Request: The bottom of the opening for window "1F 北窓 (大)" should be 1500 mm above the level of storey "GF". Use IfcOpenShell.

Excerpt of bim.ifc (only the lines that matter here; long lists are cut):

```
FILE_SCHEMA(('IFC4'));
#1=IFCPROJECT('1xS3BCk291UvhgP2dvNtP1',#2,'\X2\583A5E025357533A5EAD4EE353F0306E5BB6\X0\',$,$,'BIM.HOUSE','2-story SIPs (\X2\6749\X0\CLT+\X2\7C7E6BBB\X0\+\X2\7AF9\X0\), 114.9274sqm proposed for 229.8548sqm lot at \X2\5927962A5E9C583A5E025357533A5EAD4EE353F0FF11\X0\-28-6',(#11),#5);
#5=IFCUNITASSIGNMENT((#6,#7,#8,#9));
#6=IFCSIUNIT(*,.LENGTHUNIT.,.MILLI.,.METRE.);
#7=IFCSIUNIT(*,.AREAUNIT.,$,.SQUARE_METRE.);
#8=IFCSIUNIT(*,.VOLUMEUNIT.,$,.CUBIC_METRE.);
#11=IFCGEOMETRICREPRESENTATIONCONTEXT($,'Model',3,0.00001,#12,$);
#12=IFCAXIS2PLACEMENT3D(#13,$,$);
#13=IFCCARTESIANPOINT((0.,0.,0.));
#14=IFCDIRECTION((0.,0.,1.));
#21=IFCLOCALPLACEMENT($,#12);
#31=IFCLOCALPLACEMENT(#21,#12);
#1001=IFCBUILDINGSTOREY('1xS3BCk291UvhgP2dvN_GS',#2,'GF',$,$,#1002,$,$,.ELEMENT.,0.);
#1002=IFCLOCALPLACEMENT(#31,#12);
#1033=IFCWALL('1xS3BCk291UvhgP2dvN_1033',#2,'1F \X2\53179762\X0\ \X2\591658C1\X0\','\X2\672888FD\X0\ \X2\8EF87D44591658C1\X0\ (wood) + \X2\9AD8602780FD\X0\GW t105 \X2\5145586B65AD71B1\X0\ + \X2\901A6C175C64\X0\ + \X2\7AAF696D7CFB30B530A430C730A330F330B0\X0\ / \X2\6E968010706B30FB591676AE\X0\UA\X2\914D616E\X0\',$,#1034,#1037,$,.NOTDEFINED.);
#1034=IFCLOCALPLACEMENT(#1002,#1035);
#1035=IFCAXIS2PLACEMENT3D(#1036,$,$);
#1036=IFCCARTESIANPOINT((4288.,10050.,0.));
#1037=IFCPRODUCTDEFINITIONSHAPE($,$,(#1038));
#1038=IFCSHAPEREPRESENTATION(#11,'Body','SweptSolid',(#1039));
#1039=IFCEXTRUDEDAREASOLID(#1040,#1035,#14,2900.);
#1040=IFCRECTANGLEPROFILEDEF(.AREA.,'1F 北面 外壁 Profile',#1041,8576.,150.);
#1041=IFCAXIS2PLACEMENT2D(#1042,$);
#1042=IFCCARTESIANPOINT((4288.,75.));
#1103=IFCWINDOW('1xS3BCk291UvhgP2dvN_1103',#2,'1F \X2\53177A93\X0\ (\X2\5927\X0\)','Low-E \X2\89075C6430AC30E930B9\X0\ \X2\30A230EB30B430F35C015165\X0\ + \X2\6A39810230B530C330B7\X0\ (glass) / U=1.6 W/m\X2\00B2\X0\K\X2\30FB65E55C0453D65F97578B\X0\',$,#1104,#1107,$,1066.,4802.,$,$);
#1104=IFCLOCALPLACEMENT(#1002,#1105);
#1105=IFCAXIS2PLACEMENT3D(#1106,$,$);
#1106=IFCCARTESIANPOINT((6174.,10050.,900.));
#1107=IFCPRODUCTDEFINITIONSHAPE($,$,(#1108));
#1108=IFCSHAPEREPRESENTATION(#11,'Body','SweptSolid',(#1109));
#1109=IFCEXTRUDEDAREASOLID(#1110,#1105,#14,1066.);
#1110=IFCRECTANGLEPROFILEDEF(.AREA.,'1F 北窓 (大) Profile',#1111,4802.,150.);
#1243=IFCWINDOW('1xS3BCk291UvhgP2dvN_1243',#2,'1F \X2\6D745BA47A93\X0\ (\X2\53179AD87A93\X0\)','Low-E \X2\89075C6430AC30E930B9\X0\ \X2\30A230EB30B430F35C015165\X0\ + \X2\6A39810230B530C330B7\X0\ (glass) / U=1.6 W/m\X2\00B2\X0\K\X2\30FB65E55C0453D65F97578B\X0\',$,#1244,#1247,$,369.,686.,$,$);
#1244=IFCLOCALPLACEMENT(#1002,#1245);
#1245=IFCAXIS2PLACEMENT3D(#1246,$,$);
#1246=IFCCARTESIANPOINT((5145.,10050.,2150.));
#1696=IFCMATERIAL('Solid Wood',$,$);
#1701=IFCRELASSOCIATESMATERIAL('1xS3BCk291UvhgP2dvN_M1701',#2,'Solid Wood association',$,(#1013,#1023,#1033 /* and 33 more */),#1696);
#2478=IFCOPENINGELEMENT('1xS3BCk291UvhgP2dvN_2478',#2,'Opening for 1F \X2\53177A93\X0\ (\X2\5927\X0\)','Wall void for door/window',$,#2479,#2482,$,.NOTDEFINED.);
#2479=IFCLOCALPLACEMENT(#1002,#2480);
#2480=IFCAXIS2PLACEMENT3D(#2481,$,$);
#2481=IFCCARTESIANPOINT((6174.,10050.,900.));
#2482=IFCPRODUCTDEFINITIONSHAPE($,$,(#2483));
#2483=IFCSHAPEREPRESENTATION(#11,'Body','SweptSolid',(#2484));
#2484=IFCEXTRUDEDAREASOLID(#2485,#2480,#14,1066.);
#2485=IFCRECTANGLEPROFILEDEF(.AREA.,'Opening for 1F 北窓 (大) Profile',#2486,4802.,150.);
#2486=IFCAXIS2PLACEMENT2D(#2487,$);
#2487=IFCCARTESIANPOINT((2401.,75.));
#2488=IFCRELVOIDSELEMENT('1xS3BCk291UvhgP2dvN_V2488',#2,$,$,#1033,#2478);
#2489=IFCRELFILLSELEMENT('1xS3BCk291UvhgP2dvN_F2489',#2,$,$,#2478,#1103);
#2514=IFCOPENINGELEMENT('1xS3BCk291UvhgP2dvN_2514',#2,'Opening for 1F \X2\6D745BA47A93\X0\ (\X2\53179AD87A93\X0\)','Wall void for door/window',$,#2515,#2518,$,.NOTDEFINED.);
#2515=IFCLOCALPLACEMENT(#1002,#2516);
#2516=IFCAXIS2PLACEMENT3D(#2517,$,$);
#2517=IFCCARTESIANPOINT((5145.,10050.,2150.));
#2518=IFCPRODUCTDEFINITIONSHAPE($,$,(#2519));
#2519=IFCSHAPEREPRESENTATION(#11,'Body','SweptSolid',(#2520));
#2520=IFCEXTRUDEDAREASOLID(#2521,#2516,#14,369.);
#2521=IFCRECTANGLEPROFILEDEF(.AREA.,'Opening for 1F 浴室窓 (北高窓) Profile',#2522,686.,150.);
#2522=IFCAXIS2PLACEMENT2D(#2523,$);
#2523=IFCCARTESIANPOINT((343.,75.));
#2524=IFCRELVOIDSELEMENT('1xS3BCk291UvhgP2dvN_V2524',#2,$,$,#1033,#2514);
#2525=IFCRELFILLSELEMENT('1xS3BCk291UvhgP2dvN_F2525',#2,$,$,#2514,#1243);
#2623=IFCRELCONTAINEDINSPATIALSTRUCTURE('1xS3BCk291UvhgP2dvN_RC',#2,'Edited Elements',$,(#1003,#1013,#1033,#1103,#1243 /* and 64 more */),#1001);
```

```python
import numpy as np
import ifcopenshell
import ifcopenshell.api.geometry
import ifcopenshell.geom
import ifcopenshell.util.element
import ifcopenshell.util.placement
import ifcopenshell.util.shape
import ifcopenshell.util.unit

model = ifcopenshell.open("bim.ifc")
unit_scale = ifcopenshell.util.unit.calculate_unit_scale(model)

window = model.by_guid("1xS3BCk291UvhgP2dvN_1103")
opening = window.FillsVoids[0].RelatingOpeningElement
storey = ifcopenshell.util.element.get_container(window, ifc_class="IfcBuildingStorey")
level = ifcopenshell.util.placement.get_local_placement(storey.ObjectPlacement)[2, 3]

# The opening's origin need not be at the sill, so measure its lowest point.
shape = ifcopenshell.geom.create_shape(ifcopenshell.geom.settings(), opening)
bottom = ifcopenshell.util.shape.get_shape_bottom_elevation(shape, shape.geometry) / unit_scale
dz = level + 1500.0 - bottom

shift = np.array([0.0, 0.0, dz])
# The window is not placed relative to its opening, so move both.
for product in (opening, window):
    matrix = ifcopenshell.util.placement.get_local_placement(product.ObjectPlacement)
    matrix[:3, 3] += shift
    ifcopenshell.api.geometry.edit_object_placement(model, product=product, matrix=matrix, is_si=False)

print(f"moved by {dz * unit_scale:+.3f} m")

model.write("bim-out.ifc")
```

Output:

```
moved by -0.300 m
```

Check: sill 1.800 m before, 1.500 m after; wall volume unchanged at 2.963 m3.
